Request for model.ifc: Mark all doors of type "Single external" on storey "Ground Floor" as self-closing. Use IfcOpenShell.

First a look at what the model holds.

```python
import ifcopenshell
import ifcopenshell.util.element

model = ifcopenshell.open("model.ifc")
print(model.schema)
storey = next(s for s in model.by_type("IfcBuildingStorey") if s.Name == "Ground Floor")
doors = [e for e in ifcopenshell.util.element.get_decomposition(storey) if e.is_a("IfcDoor")]
seen = {}
for e in doors:
    element_type = ifcopenshell.util.element.get_type(e)
    key = (element_type.Name if element_type != e and element_type else None, ifcopenshell.util.element.get_pset(e, "Pset_DoorCommon", "SelfClosing"))
    seen[key] = seen.get(key, 0) + 1
for (name, value), count in sorted(seen.items(), key=str):
    print(count, "x", name, "|", value)
```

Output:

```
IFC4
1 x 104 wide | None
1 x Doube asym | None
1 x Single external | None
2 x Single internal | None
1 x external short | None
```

```python
import ifcopenshell
import ifcopenshell.api.pset
import ifcopenshell.util.element

model = ifcopenshell.open("model.ifc")

storey = next(s for s in model.by_type("IfcBuildingStorey") if s.Name == "Ground Floor")
doors = [e for e in ifcopenshell.util.element.get_decomposition(storey) if e.is_a("IfcDoor")]

count = 0
for e in doors:
    element_type = ifcopenshell.util.element.get_type(e)
    if element_type in (None, e) or element_type.Name != "Single external":
        continue
    # add_pset returns the element's existing set when there is one.
    pset = ifcopenshell.api.pset.add_pset(model, product=e, name="Pset_DoorCommon")
    ifcopenshell.api.pset.edit_pset(model, pset=pset, properties={"SelfClosing": True})
    count += 1

print(count, "doors updated")

model.write("model_edited.ifc")
```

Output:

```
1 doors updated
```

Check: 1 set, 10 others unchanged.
